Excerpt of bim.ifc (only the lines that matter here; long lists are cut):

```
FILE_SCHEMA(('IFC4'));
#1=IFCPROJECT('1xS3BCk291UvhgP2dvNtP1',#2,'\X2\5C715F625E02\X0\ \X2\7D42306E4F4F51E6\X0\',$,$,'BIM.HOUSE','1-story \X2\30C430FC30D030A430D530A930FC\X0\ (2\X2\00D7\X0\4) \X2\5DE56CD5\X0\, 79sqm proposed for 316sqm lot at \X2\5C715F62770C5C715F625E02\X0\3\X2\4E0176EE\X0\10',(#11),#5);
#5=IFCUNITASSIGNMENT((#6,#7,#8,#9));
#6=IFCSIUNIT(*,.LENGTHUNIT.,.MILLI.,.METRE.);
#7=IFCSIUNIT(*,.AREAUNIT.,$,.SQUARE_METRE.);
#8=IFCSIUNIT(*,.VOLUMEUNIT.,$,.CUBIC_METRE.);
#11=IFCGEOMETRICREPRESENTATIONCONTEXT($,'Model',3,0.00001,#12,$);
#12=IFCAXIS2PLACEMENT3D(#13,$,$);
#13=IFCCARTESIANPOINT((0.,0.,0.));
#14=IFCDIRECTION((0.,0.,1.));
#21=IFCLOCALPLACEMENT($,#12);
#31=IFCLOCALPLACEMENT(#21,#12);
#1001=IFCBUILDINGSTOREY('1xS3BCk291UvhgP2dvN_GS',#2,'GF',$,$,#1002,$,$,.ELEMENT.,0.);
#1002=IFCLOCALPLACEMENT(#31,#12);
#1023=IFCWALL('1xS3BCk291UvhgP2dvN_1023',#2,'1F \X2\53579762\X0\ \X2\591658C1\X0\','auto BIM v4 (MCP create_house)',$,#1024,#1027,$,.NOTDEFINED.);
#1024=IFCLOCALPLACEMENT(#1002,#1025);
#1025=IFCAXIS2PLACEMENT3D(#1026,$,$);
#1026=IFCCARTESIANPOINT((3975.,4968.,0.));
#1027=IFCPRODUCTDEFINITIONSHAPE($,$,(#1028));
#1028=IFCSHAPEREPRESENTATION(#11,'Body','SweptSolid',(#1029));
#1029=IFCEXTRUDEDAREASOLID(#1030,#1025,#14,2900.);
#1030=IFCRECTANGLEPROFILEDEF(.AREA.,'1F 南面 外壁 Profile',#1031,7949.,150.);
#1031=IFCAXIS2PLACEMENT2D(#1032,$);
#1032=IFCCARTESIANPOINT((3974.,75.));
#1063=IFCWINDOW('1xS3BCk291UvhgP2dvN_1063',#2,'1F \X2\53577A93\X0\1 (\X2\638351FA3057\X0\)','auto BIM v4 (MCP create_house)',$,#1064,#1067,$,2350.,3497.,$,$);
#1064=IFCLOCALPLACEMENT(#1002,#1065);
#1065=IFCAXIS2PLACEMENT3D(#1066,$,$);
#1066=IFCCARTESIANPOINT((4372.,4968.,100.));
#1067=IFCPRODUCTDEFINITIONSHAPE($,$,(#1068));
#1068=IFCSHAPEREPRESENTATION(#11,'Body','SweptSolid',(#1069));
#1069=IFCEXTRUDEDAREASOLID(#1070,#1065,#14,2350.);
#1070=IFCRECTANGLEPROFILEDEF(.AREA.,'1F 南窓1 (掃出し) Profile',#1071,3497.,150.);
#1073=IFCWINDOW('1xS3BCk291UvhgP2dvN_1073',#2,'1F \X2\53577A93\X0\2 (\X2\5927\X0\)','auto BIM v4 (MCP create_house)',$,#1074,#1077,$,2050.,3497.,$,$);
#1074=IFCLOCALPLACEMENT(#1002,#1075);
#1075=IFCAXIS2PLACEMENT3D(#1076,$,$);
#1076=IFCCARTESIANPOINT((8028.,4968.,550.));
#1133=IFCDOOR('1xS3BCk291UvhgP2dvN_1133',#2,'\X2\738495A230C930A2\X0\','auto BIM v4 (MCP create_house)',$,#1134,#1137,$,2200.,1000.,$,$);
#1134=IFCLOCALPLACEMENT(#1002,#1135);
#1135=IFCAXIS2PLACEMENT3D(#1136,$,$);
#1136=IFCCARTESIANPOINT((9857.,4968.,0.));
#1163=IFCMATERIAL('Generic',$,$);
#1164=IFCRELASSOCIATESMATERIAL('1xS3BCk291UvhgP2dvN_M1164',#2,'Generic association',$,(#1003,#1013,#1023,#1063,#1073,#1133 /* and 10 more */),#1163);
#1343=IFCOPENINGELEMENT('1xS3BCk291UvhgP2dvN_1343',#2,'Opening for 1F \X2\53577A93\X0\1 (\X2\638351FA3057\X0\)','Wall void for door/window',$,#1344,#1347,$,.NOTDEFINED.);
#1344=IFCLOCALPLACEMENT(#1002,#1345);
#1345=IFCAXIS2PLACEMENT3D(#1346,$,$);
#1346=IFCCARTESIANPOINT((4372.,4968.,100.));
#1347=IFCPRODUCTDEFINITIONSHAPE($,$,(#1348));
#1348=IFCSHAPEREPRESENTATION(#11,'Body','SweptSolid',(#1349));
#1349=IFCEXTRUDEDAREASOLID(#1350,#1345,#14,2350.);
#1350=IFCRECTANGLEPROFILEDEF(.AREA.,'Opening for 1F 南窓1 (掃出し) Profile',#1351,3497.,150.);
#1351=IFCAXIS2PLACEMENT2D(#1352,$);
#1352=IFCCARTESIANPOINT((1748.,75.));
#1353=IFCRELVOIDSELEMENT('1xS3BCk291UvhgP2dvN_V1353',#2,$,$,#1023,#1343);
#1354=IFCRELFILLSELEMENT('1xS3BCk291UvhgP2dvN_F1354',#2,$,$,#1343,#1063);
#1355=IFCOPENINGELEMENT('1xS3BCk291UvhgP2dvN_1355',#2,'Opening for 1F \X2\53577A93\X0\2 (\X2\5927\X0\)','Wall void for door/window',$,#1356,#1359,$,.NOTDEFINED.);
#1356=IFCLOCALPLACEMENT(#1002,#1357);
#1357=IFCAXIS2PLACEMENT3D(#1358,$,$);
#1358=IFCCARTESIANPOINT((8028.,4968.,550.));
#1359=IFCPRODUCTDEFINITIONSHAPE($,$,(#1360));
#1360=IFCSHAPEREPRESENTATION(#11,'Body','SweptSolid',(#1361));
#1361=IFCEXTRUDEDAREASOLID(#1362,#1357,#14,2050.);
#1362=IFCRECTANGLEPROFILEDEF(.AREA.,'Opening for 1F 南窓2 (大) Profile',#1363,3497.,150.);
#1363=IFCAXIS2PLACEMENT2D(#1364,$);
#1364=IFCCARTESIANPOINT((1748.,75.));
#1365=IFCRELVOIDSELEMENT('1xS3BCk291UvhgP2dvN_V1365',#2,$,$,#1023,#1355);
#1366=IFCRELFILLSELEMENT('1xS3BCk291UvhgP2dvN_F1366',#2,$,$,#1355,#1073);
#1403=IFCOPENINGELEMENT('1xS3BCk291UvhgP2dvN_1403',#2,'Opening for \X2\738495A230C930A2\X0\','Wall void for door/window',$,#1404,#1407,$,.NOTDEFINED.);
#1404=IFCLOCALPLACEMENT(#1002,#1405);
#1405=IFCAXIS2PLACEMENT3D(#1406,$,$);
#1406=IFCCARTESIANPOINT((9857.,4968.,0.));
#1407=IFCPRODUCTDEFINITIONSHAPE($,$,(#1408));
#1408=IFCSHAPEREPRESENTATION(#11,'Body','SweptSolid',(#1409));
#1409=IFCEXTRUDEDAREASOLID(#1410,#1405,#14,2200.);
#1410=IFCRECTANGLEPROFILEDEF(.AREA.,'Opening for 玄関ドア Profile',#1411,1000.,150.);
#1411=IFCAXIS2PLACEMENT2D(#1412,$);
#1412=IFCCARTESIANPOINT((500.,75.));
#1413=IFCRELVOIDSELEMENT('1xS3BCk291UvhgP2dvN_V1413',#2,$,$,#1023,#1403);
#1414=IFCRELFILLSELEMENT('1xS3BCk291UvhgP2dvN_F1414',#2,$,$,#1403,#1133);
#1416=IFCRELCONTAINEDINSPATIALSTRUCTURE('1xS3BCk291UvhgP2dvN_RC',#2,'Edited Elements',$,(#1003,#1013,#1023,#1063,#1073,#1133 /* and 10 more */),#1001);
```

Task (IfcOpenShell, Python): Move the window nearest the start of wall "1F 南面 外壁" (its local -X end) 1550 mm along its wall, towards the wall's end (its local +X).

```python
import ifcopenshell
import ifcopenshell.api.geometry
import ifcopenshell.util.placement
import ifcopenshell.util.unit

model = ifcopenshell.open("bim.ifc")
unit_scale = ifcopenshell.util.unit.calculate_unit_scale(model)

window = model.by_id(1063)
opening = window.FillsVoids[0].RelatingOpeningElement
wall = opening.VoidsElements[0].RelatingBuildingElement

wall_matrix = ifcopenshell.util.placement.get_local_placement(wall.ObjectPlacement)
shift = wall_matrix[:3, 0] * 1.55 / unit_scale
before = ifcopenshell.util.placement.get_local_placement(window.ObjectPlacement)[:3, 3].copy()

# The window is not placed relative to its opening, so move both.
for product in (opening, window):
    matrix = ifcopenshell.util.placement.get_local_placement(product.ObjectPlacement)
    matrix[:3, 3] += shift
    ifcopenshell.api.geometry.edit_object_placement(model, product=product, matrix=matrix, is_si=False)

after = ifcopenshell.util.placement.get_local_placement(window.ObjectPlacement)[:3, 3]
print("window moved by", (after - before).round(3) + 0.0)

model.write("bim_updated.ifc")
```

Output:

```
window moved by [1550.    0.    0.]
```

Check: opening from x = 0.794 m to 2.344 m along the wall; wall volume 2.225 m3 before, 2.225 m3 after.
